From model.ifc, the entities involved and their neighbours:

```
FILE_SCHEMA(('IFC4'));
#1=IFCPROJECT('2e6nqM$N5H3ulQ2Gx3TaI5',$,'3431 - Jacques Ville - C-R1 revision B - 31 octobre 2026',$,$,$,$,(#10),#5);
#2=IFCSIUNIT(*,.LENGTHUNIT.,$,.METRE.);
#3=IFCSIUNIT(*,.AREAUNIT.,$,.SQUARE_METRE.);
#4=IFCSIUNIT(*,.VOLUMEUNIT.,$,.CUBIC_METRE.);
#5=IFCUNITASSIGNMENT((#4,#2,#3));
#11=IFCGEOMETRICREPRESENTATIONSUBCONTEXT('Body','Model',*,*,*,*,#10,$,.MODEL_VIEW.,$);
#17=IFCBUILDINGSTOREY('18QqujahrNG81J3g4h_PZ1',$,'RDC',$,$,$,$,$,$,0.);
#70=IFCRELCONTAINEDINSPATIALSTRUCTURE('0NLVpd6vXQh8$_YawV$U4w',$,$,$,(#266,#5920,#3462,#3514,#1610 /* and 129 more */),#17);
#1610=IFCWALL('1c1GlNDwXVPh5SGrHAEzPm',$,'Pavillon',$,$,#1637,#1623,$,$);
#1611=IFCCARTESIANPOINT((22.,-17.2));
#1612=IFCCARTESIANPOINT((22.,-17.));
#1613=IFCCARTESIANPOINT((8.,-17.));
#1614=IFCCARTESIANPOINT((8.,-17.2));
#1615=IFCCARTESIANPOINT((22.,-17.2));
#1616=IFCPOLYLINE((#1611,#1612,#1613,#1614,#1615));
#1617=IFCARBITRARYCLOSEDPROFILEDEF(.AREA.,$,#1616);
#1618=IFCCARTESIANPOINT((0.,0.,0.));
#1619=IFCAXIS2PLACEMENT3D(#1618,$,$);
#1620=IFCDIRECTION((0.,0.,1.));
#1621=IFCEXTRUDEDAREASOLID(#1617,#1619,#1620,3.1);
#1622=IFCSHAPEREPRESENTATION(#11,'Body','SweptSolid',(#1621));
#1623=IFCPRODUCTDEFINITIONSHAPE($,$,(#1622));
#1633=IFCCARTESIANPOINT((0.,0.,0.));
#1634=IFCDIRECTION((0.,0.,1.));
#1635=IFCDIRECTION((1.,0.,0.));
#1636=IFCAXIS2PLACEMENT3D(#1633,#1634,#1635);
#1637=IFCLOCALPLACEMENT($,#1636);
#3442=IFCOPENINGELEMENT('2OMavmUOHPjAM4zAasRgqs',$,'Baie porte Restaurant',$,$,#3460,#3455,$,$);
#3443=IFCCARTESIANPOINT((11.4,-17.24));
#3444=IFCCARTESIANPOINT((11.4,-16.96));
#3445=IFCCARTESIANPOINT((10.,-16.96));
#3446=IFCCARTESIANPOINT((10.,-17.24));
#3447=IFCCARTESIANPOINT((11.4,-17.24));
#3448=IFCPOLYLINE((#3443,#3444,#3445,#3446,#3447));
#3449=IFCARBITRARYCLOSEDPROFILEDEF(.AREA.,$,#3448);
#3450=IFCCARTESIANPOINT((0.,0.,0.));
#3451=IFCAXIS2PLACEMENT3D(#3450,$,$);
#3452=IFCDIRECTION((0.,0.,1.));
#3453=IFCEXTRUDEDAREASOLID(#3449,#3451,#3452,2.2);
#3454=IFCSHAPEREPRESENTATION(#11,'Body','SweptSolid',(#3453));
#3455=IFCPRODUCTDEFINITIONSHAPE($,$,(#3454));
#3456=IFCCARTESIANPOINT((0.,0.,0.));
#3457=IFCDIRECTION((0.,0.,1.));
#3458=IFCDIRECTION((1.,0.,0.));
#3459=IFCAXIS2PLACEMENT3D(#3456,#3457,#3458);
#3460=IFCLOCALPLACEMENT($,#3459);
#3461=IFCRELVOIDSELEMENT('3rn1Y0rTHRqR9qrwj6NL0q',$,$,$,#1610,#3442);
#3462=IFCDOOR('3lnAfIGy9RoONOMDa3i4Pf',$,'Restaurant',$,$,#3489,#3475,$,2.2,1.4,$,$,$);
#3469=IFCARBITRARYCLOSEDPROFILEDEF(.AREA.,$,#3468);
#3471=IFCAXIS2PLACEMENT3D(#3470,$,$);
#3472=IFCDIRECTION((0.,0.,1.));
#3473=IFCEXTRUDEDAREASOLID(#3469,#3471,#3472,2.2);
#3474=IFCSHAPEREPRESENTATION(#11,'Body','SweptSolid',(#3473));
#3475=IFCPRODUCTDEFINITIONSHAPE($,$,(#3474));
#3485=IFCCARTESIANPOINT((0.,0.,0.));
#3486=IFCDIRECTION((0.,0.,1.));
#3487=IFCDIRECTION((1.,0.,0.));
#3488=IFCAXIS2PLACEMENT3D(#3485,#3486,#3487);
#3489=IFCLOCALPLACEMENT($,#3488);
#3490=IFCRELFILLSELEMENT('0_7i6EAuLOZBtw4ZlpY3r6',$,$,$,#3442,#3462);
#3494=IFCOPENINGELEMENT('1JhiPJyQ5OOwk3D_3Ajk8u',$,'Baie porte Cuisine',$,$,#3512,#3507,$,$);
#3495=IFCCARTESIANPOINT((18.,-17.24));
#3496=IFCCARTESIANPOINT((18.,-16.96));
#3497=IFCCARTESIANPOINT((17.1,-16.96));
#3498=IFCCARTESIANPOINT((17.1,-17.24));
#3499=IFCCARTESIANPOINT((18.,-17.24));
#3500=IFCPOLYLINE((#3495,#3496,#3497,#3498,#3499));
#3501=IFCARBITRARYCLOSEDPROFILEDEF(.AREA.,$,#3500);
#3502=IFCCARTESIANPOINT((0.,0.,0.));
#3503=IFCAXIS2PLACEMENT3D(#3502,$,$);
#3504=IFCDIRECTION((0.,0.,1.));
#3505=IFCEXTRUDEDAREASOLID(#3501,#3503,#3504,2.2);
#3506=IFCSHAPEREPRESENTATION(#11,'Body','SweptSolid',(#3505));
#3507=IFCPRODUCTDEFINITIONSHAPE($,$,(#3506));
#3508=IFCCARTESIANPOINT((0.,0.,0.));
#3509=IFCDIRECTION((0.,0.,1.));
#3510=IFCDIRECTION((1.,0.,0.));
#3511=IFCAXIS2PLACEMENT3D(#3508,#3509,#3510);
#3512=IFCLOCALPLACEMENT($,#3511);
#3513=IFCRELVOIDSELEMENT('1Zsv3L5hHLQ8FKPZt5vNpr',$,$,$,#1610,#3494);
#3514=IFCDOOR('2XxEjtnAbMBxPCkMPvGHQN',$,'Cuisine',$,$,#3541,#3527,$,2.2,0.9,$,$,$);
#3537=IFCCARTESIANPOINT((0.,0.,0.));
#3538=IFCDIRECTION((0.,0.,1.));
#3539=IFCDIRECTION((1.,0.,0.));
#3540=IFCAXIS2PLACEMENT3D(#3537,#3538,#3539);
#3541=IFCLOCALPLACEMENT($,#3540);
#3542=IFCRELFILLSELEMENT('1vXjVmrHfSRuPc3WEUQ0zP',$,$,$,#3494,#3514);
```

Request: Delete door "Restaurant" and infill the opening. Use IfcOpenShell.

```python
import ifcopenshell
import ifcopenshell.api.feature
import ifcopenshell.api.root
import ifcopenshell.geom
import ifcopenshell.util.shape

model = ifcopenshell.open("model.ifc")
settings = ifcopenshell.geom.settings()


def volume(element):
    """Net volume in cubic metres, openings subtracted."""
    shape = ifcopenshell.geom.create_shape(settings, element)
    return ifcopenshell.util.shape.get_volume(shape.geometry)


door = model.by_id(3462)
opening = door.FillsVoids[0].RelatingOpeningElement
wall = opening.VoidsElements[0].RelatingBuildingElement
before = volume(wall)

ifcopenshell.api.root.remove_product(model, product=door)
ifcopenshell.api.feature.remove_feature(model, feature=opening)

after = volume(wall)

print(f"wall volume {before:.3f} -> {after:.3f} m3")

model.write("model_v2.ifc")
```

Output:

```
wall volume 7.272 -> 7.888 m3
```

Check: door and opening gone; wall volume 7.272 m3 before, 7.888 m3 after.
